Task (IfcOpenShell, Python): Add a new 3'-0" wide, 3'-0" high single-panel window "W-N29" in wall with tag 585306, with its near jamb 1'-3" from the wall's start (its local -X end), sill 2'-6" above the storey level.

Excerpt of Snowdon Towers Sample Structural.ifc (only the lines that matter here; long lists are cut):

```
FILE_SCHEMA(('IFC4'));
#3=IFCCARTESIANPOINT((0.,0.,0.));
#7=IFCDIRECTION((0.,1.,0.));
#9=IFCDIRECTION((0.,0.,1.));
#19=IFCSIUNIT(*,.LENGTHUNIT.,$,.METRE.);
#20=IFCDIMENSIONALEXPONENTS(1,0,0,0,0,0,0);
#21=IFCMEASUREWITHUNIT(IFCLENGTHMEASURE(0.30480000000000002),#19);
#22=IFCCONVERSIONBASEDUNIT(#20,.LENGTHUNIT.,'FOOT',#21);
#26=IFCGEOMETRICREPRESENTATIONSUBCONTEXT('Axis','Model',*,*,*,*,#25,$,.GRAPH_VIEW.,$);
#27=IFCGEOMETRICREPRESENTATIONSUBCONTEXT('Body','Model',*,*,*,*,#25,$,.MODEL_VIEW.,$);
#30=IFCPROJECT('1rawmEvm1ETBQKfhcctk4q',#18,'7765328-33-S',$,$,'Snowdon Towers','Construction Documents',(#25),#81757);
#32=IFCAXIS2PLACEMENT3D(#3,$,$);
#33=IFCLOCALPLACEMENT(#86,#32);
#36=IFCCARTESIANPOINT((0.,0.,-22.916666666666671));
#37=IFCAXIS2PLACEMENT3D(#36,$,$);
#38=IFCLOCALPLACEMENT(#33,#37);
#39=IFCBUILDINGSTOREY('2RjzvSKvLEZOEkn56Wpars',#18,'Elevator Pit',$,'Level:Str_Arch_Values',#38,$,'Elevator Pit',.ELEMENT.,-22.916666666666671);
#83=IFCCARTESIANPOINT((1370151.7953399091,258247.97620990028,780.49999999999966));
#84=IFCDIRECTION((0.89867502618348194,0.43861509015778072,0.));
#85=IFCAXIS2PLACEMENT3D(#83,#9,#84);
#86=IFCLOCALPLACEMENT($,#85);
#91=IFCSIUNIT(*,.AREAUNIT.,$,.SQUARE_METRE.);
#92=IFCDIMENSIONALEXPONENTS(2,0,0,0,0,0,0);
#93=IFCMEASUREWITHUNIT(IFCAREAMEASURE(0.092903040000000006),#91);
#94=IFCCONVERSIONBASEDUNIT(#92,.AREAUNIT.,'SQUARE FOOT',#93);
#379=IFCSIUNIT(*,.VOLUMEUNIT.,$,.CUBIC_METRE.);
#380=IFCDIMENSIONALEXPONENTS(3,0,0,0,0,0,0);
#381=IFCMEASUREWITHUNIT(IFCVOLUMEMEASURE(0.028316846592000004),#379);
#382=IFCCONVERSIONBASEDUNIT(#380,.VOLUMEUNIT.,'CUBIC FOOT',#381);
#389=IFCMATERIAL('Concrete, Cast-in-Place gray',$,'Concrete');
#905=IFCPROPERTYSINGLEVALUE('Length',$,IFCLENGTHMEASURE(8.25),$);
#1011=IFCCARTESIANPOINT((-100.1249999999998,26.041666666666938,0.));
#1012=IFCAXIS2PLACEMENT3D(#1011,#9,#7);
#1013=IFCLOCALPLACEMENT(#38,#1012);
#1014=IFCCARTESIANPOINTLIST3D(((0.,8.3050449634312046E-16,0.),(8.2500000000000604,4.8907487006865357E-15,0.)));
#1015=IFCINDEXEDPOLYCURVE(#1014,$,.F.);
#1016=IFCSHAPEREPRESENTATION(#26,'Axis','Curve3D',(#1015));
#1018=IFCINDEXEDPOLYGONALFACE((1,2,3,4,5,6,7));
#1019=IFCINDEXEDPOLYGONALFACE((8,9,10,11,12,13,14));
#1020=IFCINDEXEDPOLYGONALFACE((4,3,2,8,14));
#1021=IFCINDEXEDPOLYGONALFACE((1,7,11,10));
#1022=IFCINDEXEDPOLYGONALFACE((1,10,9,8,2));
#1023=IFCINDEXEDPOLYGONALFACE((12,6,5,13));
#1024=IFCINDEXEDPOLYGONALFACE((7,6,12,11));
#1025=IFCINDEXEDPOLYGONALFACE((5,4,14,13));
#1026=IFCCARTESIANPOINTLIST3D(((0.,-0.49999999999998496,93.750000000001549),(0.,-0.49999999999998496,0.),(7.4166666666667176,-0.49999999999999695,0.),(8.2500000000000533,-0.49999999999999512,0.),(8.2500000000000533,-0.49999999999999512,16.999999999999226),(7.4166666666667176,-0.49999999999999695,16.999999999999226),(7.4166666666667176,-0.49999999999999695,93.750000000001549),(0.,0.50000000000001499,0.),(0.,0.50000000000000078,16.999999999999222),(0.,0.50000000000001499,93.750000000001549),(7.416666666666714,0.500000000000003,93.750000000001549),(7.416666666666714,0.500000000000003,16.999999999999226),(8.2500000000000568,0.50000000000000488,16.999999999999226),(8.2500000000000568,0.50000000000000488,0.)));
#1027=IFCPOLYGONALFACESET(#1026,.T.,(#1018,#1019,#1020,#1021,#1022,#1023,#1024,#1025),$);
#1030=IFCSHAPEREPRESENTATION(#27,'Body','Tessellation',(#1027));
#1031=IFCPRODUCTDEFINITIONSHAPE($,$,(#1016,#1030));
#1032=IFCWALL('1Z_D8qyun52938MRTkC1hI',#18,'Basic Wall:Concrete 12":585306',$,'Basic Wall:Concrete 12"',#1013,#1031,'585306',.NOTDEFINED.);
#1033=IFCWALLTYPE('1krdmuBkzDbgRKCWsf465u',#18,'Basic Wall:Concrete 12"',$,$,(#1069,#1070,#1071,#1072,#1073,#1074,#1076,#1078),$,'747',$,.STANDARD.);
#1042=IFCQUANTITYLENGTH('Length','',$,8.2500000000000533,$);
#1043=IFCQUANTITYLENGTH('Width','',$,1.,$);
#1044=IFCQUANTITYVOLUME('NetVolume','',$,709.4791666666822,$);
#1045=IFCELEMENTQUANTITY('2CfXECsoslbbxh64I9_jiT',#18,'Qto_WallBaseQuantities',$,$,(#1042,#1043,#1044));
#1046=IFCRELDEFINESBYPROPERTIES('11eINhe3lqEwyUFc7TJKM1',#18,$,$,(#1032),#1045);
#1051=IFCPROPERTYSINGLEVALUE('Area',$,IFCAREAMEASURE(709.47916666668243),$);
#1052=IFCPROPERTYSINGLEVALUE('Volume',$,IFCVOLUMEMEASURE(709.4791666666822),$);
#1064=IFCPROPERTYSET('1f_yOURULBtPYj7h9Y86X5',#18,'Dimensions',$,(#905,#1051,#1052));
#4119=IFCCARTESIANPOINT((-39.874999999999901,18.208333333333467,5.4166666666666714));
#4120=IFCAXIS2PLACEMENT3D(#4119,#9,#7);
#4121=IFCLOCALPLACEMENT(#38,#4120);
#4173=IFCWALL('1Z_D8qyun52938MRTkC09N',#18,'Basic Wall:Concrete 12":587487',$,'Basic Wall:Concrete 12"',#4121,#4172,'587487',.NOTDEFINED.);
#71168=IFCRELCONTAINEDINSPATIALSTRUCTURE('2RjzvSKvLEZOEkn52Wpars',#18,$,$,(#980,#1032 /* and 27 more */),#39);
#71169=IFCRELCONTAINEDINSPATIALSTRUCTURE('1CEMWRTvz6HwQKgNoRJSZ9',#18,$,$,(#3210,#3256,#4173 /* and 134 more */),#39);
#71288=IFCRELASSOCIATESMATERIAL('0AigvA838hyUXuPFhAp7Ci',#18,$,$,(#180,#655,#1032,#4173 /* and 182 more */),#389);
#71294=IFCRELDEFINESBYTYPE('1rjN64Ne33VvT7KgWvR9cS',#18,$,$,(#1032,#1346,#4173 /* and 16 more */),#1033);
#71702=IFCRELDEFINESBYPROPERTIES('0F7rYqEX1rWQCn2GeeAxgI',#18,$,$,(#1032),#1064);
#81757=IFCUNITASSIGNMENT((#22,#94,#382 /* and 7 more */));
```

```python
import numpy as np
import ifcopenshell
import ifcopenshell.api.feature
import ifcopenshell.api.geometry
import ifcopenshell.api.pset
import ifcopenshell.api.root
import ifcopenshell.api.spatial
import ifcopenshell.geom
import ifcopenshell.util.element
import ifcopenshell.util.placement
import ifcopenshell.util.representation
import ifcopenshell.util.shape
import ifcopenshell.util.unit

model = ifcopenshell.open("Snowdon Towers Sample Structural.ifc")
unit_scale = ifcopenshell.util.unit.calculate_unit_scale(model)
area_scale = ifcopenshell.util.unit.calculate_unit_scale(model, "AREAUNIT")
volume_scale = ifcopenshell.util.unit.calculate_unit_scale(model, "VOLUMEUNIT")
settings = ifcopenshell.geom.settings()


def volume(element):
    """Net volume in cubic metres, openings subtracted."""
    shape = ifcopenshell.geom.create_shape(settings, element)
    return ifcopenshell.util.shape.get_volume(shape.geometry)


wall = model.by_guid("1Z_D8qyun52938MRTkC1hI")
storey = ifcopenshell.util.element.get_container(wall, ifc_class="IfcBuildingStorey")
context = ifcopenshell.util.representation.get_context(model, "Model", "Body", "MODEL_VIEW")
before = volume(wall)

width, height, from_end, sill = 0.9144, 0.9144, 0.381, 0.762  # metres

# The wall runs along its own X axis, and the end named is its -X end.
wall_shape = ifcopenshell.geom.create_shape(settings, wall)
x, y, z = ifcopenshell.util.shape.get_vertices(wall_shape.geometry).T
start = x.min() + from_end
face, thickness = float(y.min()), float(y.max() - y.min())
wall_matrix = ifcopenshell.util.placement.get_local_placement(wall.ObjectPlacement)
level = ifcopenshell.util.placement.get_local_placement(storey.ObjectPlacement)[2, 3]


def in_wall(x, y):
    """Placement at x, y metres in the wall's axes, at sill height."""
    matrix = wall_matrix.copy()
    matrix[:, 3] = wall_matrix @ np.array([x / unit_scale, y / unit_scale, 0.0, 1.0])
    matrix[2, 3] = level + sill / unit_scale
    return matrix


# Opening: a box that overshoots both wall faces by 50 mm.
opening = ifcopenshell.api.root.create_entity(model, ifc_class="IfcOpeningElement", predefined_type="OPENING")
box = ifcopenshell.api.geometry.add_wall_representation(
    model, context=context, length=width, height=height, thickness=thickness + 0.1
)
ifcopenshell.api.geometry.assign_representation(model, product=opening, representation=box)
ifcopenshell.api.geometry.edit_object_placement(model, product=opening, matrix=in_wall(start, face - 0.05), is_si=False)
ifcopenshell.api.feature.add_feature(model, feature=opening, element=wall)

window = ifcopenshell.api.root.create_entity(model, ifc_class="IfcWindow", name="W-N29", predefined_type="WINDOW")
window.OverallWidth, window.OverallHeight = width / unit_scale, height / unit_scale
window.PartitioningType = "SINGLE_PANEL"
body = ifcopenshell.api.geometry.add_window_representation(
    model,
    context=context,
    overall_width=window.OverallWidth,
    overall_height=window.OverallHeight,
    partition_type="SINGLE_PANEL",
)
ifcopenshell.api.geometry.assign_representation(model, product=window, representation=body)
ifcopenshell.api.spatial.assign_container(model, products=[window], relating_structure=storey)
ifcopenshell.api.feature.add_filling(model, opening=opening, element=window)

# Centre the window in the wall's thickness.
ifcopenshell.api.geometry.edit_object_placement(model, product=window, matrix=in_wall(start, face), is_si=False)
window_shape = ifcopenshell.geom.create_shape(settings, window)
depth = ifcopenshell.util.shape.get_vertices(window_shape.geometry)[:, 1]
offset = face + thickness / 2 - (depth.min() + depth.max()) / 2
ifcopenshell.api.geometry.edit_object_placement(model, product=window, matrix=in_wall(start, offset), is_si=False)

after = volume(wall)

# Update the wall's stored quantities.
qto = model.by_id(ifcopenshell.util.element.get_pset(wall, "Qto_WallBaseQuantities", should_inherit=False)["id"])
ifcopenshell.api.pset.edit_qto(model, qto=qto, properties={"NetVolume": after / volume_scale})
pset = model.by_id(ifcopenshell.util.element.get_pset(wall, "Dimensions", should_inherit=False)["id"])
ifcopenshell.api.pset.edit_pset(model, pset=pset, properties={
    "Area": model.create_entity("IfcAreaMeasure", after / thickness / area_scale),
    "Volume": model.create_entity("IfcVolumeMeasure", after / volume_scale),
})

print(f"wall volume {before:.3f} -> {after:.3f} m3")

model.write("Snowdon Towers Sample Structural_v2.ifc")
```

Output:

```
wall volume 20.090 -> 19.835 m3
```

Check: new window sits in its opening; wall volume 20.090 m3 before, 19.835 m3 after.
